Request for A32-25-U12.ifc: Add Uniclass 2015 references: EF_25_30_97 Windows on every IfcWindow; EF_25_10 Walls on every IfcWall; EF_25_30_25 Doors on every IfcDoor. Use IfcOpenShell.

First a look at what the model holds.

```python
import ifcopenshell

model = ifcopenshell.open("A32-25-U12.ifc")
print(model.schema)
print("classifications:", [c.Name for c in model.by_type("IfcClassification")])
for ifc_class in ("IfcDoor", "IfcRoof", "IfcStair", "IfcWall", "IfcWindow"):
    print(ifc_class, len(model.by_type(ifc_class)))
```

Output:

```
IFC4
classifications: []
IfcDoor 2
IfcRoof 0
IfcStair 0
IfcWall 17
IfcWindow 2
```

```python
import ifcopenshell
import ifcopenshell.api.classification

model = ifcopenshell.open("A32-25-U12.ifc")

system = ifcopenshell.api.classification.add_classification(model, classification="Uniclass 2015")

codes = {
    "IfcWindow": ("EF_25_30_97", "Windows"),
    "IfcWall": ("EF_25_10", "Walls"),
    "IfcDoor": ("EF_25_30_25", "Doors"),
}
for ifc_class, (code, name) in codes.items():
    products = model.by_type(ifc_class)
    ifcopenshell.api.classification.add_reference(
        model, products=products, classification=system, identification=code, name=name
    )
    print(code, len(products))

model.write("A32-25-U12_updated.ifc")
```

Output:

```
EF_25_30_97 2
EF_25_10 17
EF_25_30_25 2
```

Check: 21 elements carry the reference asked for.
